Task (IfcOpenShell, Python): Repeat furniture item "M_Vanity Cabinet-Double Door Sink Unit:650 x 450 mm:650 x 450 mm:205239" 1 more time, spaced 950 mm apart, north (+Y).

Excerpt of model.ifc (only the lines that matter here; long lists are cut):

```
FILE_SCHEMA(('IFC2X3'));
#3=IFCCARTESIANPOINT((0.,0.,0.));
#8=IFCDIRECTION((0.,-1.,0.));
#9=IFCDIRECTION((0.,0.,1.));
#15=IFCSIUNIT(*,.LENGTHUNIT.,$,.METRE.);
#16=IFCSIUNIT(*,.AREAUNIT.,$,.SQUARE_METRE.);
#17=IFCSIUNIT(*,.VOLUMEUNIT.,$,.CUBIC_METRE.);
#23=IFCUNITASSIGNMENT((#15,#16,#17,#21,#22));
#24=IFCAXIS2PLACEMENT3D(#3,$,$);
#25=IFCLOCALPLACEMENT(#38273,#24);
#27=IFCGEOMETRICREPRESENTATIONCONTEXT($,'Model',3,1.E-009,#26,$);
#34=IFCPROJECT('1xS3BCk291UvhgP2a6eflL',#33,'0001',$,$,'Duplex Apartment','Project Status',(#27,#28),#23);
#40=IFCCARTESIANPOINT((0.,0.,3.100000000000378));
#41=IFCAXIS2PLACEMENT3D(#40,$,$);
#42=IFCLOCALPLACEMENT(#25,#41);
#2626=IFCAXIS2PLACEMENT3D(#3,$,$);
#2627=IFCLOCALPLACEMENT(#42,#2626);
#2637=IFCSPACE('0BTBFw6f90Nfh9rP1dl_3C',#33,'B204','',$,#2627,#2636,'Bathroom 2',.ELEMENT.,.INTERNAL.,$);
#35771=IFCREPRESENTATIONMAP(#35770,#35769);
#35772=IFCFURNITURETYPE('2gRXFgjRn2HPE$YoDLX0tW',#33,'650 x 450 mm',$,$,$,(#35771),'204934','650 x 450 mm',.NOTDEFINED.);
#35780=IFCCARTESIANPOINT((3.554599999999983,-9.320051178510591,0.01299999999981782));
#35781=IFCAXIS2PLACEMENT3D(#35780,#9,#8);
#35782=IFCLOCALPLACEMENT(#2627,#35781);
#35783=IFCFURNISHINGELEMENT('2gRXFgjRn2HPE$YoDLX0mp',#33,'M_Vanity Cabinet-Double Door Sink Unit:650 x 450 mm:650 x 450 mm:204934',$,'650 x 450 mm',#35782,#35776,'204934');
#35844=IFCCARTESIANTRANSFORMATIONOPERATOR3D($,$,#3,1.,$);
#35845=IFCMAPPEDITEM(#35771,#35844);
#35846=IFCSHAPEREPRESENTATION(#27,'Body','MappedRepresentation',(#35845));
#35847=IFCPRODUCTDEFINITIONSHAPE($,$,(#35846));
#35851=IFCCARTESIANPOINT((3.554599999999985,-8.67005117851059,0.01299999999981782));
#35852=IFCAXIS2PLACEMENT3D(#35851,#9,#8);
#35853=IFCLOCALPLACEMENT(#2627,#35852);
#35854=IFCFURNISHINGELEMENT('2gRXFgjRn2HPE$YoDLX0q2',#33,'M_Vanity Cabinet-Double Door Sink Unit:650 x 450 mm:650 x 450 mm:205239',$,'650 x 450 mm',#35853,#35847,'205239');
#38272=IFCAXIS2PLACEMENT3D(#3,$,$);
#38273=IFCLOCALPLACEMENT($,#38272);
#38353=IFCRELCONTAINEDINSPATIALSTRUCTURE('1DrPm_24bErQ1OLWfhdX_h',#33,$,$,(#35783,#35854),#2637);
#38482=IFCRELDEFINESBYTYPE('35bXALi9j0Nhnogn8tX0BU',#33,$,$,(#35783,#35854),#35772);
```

```python
import numpy as np
import ifcopenshell
import ifcopenshell.api.geometry
import ifcopenshell.api.root
import ifcopenshell.util.element
import ifcopenshell.util.placement

model = ifcopenshell.open("model.ifc")


def reuse_history(source, copy):
    """copy_class also copies each property set's owner history, people and application; keep the originals."""
    for rel in copy.IsDefinedBy:
        if rel.is_a("IfcRelDefinesByProperties") and (history := rel.RelatingPropertyDefinition.OwnerHistory):
            rel.RelatingPropertyDefinition.OwnerHistory = source.OwnerHistory
            ifcopenshell.util.element.remove_deep2(model, history)


source = model.by_guid("2gRXFgjRn2HPE$YoDLX0q2")
base = ifcopenshell.util.placement.get_local_placement(source.ObjectPlacement)
step = np.array([0.0, 1.0, 0.0]) * 0.95

for i in range(1, 2):
    copy = ifcopenshell.api.root.copy_class(model, product=source)
    copy.Representation = ifcopenshell.util.element.copy_deep(
        model, source.Representation, exclude=["IfcGeometricRepresentationContext", "IfcRepresentationMap"]
    )
    copy.Name = "M_Vanity Cabinet-Double Door Sink Unit:650 x 450 mm:650 x 450 mm"
    copy.Tag = None
    reuse_history(source, copy)
    matrix = base.copy()
    matrix[:3, 3] += i * step
    print("added at", matrix[:3, 3].round(3) + 0.0)
    ifcopenshell.api.geometry.edit_object_placement(model, product=copy, matrix=matrix, is_si=False)

model.write("model-out.ifc")
```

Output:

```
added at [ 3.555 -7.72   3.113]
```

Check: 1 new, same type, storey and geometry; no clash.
